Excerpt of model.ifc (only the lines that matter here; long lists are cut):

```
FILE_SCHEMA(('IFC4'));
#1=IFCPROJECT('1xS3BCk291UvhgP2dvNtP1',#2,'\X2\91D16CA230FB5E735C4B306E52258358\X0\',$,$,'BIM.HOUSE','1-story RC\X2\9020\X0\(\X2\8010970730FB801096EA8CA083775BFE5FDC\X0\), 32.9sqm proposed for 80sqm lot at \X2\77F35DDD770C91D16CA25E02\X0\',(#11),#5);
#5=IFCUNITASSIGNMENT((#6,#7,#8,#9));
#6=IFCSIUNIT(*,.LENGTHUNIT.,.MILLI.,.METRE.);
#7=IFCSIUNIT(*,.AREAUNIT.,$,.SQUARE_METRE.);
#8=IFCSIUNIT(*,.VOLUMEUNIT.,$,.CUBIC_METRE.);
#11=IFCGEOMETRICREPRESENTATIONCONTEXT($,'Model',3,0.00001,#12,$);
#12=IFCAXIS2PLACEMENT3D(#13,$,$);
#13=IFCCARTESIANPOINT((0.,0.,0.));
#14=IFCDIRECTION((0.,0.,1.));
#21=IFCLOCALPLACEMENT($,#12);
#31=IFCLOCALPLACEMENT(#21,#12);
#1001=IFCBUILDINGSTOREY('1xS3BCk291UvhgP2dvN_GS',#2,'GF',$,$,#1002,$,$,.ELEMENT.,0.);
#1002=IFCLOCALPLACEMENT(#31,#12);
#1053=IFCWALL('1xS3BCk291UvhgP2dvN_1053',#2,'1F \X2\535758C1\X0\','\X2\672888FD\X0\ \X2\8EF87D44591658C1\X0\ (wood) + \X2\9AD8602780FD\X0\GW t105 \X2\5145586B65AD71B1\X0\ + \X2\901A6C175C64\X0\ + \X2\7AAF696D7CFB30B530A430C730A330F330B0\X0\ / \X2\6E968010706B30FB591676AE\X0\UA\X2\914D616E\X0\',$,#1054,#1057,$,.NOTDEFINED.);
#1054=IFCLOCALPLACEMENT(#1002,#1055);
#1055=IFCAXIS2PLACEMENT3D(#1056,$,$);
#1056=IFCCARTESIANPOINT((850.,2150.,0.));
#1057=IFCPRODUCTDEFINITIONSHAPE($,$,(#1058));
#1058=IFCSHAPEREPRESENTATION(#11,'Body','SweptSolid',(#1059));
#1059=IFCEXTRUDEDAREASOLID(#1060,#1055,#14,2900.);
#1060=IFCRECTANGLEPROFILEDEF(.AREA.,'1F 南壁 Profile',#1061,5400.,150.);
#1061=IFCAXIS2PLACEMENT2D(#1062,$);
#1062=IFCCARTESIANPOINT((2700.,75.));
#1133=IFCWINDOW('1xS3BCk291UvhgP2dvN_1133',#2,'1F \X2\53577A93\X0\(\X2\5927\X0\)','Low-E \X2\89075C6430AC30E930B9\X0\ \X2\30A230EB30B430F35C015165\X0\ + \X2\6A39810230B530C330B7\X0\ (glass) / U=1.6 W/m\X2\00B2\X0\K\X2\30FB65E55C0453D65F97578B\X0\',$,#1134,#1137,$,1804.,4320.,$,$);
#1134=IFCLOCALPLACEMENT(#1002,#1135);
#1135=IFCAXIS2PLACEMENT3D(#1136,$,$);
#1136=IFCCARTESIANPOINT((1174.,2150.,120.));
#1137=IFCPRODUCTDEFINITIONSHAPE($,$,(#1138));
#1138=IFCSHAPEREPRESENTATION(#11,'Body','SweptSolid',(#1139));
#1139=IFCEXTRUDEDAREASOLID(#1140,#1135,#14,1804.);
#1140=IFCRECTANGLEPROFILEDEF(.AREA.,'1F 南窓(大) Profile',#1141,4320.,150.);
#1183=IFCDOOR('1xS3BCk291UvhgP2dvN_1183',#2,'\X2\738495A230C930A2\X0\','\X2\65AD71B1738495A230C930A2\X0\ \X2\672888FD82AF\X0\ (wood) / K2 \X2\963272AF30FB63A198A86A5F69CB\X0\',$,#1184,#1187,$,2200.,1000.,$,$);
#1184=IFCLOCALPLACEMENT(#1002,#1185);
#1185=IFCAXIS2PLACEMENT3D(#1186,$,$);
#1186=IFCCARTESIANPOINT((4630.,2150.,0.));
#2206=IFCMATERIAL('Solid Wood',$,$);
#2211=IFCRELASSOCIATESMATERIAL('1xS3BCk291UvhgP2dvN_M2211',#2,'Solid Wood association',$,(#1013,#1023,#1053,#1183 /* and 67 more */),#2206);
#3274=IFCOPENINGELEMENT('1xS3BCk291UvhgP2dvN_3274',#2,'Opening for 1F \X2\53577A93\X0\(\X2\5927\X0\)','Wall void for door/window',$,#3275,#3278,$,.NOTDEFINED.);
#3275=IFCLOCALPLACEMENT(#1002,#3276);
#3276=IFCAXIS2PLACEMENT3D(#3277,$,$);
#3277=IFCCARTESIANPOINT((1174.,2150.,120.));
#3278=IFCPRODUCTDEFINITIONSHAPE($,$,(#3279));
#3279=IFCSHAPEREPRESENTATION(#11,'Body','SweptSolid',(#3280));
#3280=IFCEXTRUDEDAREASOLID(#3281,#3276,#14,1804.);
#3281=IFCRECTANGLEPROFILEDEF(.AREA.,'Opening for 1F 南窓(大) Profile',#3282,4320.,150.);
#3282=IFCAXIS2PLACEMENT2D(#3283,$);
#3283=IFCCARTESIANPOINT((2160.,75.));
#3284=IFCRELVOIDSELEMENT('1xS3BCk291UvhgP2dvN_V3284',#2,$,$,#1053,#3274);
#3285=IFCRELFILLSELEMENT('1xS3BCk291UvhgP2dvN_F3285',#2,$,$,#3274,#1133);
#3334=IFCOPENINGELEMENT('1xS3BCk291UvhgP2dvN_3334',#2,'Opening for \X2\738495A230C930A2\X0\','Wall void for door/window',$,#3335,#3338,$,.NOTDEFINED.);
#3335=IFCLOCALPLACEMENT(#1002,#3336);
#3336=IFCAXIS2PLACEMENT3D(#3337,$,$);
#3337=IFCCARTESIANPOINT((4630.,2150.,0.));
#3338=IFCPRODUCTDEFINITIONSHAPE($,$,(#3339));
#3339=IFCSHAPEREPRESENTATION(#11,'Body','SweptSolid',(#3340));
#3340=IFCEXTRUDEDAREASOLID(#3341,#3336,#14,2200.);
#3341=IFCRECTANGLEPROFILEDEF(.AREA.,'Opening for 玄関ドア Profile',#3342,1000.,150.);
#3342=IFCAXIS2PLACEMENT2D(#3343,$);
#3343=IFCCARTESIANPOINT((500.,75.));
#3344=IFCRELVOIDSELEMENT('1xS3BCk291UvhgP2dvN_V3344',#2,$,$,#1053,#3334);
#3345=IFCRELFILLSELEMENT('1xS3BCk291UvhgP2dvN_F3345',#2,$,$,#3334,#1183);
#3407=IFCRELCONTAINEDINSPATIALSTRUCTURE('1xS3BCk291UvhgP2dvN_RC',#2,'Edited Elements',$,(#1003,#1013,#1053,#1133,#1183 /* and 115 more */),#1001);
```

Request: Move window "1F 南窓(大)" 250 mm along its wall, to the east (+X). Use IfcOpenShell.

```python
import ifcopenshell
import ifcopenshell.api.geometry
import ifcopenshell.util.placement
import ifcopenshell.util.unit

model = ifcopenshell.open("model.ifc")
unit_scale = ifcopenshell.util.unit.calculate_unit_scale(model)

window = model.by_id(1133)
opening = window.FillsVoids[0].RelatingOpeningElement
wall = opening.VoidsElements[0].RelatingBuildingElement

wall_matrix = ifcopenshell.util.placement.get_local_placement(wall.ObjectPlacement)
shift = wall_matrix[:3, 0] * 0.25 / unit_scale
before = ifcopenshell.util.placement.get_local_placement(window.ObjectPlacement)[:3, 3].copy()

# The window is not placed relative to its opening, so move both.
for product in (opening, window):
    matrix = ifcopenshell.util.placement.get_local_placement(product.ObjectPlacement)
    matrix[:3, 3] += shift
    ifcopenshell.api.geometry.edit_object_placement(model, product=product, matrix=matrix, is_si=False)

after = ifcopenshell.util.placement.get_local_placement(window.ObjectPlacement)[:3, 3]
print("window moved by", (after - before).round(3) + 0.0)

model.write("model_updated.ifc")
```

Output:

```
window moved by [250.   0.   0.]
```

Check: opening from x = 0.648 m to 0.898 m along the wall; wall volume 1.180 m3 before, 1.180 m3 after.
